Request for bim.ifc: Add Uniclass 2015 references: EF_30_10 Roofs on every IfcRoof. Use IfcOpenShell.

First a look at what the model holds.

```python
import ifcopenshell

model = ifcopenshell.open("bim.ifc")
print(model.schema)
print("classifications:", [c.Name for c in model.by_type("IfcClassification")])
for ifc_class in ("IfcDoor", "IfcRoof", "IfcStair", "IfcWall", "IfcWindow"):
    print(ifc_class, len(model.by_type(ifc_class)))
```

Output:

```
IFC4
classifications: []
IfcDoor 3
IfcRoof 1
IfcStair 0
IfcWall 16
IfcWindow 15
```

```python
import ifcopenshell
import ifcopenshell.api.classification

model = ifcopenshell.open("bim.ifc")

system = ifcopenshell.api.classification.add_classification(model, classification="Uniclass 2015")

codes = {
    "IfcRoof": ("EF_30_10", "Roofs"),
}
for ifc_class, (code, name) in codes.items():
    products = model.by_type(ifc_class)
    ifcopenshell.api.classification.add_reference(
        model, products=products, classification=system, identification=code, name=name
    )
    print(code, len(products))

model.write("bim_rev.ifc")
```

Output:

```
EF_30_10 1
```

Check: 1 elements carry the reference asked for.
